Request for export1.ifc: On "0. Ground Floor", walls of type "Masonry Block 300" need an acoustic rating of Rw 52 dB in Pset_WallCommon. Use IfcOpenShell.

First a look at what the model holds.

```python
import ifcopenshell
import ifcopenshell.util.element

model = ifcopenshell.open("export1.ifc")
print(model.schema)
storey = next(s for s in model.by_type("IfcBuildingStorey") if s.Name == "0. Ground Floor")
walls = [e for e in ifcopenshell.util.element.get_decomposition(storey) if e.is_a("IfcWall")]
seen = {}
for e in walls:
    element_type = ifcopenshell.util.element.get_type(e)
    key = (element_type.Name if element_type != e and element_type else None, ifcopenshell.util.element.get_pset(e, "Pset_WallCommon", "AcousticRating"))
    seen[key] = seen.get(key, 0) + 1
for (name, value), count in sorted(seen.items(), key=str):
    print(count, "x", name, "|", value)
```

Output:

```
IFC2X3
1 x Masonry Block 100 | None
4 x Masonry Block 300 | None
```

```python
import ifcopenshell
import ifcopenshell.api.pset
import ifcopenshell.util.element

model = ifcopenshell.open("export1.ifc")

storey = next(s for s in model.by_type("IfcBuildingStorey") if s.Name == "0. Ground Floor")
walls = [e for e in ifcopenshell.util.element.get_decomposition(storey) if e.is_a("IfcWall")]

count = 0
for e in walls:
    element_type = ifcopenshell.util.element.get_type(e)
    if element_type in (None, e) or element_type.Name != "Masonry Block 300":
        continue
    # add_pset returns the element's existing set when there is one.
    pset = ifcopenshell.api.pset.add_pset(model, product=e, name="Pset_WallCommon")
    ifcopenshell.api.pset.edit_pset(model, pset=pset, properties={"AcousticRating": "Rw 52 dB"})
    count += 1

print(count, "walls updated")

model.write("export1-out.ifc")
```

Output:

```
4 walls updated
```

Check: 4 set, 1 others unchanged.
